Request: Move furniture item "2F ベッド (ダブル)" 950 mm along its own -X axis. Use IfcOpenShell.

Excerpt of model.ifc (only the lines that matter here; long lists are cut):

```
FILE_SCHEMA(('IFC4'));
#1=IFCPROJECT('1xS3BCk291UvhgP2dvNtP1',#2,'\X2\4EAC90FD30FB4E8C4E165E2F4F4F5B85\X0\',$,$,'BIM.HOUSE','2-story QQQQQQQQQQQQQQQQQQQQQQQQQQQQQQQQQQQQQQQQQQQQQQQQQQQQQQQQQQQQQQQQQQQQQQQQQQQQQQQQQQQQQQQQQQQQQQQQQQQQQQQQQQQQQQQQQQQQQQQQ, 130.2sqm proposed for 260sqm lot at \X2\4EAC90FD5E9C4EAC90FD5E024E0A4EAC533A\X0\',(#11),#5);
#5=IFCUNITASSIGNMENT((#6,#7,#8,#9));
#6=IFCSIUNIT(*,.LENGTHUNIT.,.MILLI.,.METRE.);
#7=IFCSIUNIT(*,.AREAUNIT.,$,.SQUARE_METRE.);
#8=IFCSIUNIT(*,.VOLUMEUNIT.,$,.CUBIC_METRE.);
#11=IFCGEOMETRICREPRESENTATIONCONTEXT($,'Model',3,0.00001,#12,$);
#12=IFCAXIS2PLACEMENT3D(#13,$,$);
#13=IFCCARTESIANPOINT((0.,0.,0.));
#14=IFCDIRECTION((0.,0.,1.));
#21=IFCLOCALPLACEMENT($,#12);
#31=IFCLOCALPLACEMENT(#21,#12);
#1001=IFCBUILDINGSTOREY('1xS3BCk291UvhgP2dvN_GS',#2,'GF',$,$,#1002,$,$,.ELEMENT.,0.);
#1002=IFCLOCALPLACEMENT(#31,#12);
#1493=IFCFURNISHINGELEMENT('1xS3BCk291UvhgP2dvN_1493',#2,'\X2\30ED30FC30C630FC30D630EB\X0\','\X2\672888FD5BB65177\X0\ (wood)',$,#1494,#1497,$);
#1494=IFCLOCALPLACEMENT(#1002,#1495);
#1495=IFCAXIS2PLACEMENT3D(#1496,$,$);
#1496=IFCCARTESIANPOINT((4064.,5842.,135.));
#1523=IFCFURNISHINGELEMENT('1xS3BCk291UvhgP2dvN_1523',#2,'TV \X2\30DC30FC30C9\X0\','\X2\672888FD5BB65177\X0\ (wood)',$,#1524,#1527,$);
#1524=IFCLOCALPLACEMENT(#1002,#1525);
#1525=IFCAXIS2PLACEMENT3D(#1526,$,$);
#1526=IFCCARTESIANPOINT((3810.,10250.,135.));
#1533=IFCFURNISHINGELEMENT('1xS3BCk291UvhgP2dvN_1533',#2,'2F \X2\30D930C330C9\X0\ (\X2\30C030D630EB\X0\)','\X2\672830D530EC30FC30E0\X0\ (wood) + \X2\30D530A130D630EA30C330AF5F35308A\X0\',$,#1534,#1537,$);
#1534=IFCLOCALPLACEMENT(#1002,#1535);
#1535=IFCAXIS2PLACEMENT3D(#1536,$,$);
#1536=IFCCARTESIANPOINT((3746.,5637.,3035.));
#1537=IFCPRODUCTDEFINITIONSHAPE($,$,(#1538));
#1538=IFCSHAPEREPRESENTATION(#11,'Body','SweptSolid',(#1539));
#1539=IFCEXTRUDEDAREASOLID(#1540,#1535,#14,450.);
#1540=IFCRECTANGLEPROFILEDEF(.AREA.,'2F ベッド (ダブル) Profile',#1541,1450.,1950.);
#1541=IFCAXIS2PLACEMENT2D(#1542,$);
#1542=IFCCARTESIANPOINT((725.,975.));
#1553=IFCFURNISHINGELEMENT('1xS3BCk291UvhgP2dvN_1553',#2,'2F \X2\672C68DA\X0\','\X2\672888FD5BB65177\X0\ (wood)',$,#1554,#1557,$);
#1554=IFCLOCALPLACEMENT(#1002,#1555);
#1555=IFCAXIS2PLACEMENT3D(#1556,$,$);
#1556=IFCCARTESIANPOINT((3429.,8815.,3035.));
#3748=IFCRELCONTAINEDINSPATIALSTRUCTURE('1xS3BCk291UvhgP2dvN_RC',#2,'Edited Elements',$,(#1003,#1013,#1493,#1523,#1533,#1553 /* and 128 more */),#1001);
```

```python
import ifcopenshell
import ifcopenshell.api.geometry
import ifcopenshell.util.placement
import ifcopenshell.util.unit

model = ifcopenshell.open("model.ifc")
unit_scale = ifcopenshell.util.unit.calculate_unit_scale(model)

item = model.by_guid("1xS3BCk291UvhgP2dvN_1533")
matrix = ifcopenshell.util.placement.get_local_placement(item.ObjectPlacement)
matrix[:3, 3] -= matrix[:3, 0] * 0.95 / unit_scale
ifcopenshell.api.geometry.edit_object_placement(model, product=item, matrix=matrix, is_si=False)

print(ifcopenshell.util.placement.get_local_placement(item.ObjectPlacement).round(3) + 0.0)

model.write("model_edited.ifc")
```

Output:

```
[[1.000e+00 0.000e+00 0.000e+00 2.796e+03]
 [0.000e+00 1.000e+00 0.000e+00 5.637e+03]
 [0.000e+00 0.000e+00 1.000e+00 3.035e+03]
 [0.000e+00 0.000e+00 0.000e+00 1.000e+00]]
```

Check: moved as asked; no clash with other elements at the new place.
